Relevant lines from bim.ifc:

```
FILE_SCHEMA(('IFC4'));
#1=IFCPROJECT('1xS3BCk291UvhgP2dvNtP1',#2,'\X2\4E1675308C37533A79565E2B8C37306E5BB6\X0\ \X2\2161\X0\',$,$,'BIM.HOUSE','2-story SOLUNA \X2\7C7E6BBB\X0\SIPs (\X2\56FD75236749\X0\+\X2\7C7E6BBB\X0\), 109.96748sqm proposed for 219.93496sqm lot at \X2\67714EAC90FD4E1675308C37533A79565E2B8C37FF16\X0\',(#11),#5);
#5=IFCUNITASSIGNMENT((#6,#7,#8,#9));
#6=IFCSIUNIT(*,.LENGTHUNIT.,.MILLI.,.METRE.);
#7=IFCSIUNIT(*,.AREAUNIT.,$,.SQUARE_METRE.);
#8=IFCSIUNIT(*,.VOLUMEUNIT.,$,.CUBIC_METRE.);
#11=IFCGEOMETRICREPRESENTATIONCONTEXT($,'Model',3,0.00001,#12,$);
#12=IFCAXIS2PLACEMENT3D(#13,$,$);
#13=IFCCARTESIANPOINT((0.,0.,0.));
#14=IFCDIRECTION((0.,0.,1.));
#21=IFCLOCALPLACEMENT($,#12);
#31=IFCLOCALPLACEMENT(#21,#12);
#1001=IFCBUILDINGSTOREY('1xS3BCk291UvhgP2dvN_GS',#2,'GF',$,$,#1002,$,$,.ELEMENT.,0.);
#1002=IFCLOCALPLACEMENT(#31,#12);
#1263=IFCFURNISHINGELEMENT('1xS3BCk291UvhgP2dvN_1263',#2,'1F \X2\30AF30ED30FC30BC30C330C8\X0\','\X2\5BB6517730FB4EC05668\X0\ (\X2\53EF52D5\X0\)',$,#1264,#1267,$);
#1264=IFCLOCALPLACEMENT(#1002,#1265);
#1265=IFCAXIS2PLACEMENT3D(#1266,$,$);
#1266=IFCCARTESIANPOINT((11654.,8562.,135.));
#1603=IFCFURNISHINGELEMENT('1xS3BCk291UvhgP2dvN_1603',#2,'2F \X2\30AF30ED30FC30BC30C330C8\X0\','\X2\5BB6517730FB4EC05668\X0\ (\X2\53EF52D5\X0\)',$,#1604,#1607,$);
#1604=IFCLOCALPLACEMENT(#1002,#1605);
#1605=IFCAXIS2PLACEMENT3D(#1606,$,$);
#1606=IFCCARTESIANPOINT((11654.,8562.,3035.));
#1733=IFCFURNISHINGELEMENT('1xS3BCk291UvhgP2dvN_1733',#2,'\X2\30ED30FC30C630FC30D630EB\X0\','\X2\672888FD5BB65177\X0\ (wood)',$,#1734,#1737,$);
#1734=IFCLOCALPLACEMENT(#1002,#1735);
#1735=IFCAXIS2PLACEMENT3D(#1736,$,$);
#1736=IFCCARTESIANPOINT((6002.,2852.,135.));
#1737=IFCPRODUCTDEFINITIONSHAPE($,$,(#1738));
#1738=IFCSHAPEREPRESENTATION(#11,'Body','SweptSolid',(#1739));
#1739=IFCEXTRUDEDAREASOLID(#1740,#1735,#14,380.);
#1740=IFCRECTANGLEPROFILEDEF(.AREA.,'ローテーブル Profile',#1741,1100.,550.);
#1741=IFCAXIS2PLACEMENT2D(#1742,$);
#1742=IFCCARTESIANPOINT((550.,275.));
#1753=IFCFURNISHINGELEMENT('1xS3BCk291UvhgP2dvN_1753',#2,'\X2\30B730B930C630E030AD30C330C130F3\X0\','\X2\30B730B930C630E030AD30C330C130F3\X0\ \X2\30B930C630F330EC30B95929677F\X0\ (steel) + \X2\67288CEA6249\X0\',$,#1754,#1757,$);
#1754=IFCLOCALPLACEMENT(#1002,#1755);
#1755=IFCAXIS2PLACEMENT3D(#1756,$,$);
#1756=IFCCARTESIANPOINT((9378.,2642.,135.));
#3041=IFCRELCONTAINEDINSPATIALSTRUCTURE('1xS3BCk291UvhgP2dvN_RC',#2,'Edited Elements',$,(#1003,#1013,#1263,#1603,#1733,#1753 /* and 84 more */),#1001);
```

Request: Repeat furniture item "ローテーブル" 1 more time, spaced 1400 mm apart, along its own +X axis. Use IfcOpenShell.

```python
import ifcopenshell
import ifcopenshell.api.geometry
import ifcopenshell.api.root
import ifcopenshell.util.element
import ifcopenshell.util.placement
import ifcopenshell.util.unit

model = ifcopenshell.open("bim.ifc")
unit_scale = ifcopenshell.util.unit.calculate_unit_scale(model)


def reuse_history(source, copy):
    """copy_class also copies each property set's owner history, people and application; keep the originals."""
    for rel in copy.IsDefinedBy:
        if rel.is_a("IfcRelDefinesByProperties") and (history := rel.RelatingPropertyDefinition.OwnerHistory):
            rel.RelatingPropertyDefinition.OwnerHistory = source.OwnerHistory
            ifcopenshell.util.element.remove_deep2(model, history)


source = model.by_id(1733)
base = ifcopenshell.util.placement.get_local_placement(source.ObjectPlacement)
step = base[:3, 0] * 1.4 / unit_scale

for i in range(1, 2):
    copy = ifcopenshell.api.root.copy_class(model, product=source)
    copy.Representation = ifcopenshell.util.element.copy_deep(
        model, source.Representation, exclude=["IfcGeometricRepresentationContext", "IfcRepresentationMap"]
    )
    reuse_history(source, copy)
    matrix = base.copy()
    matrix[:3, 3] += i * step
    print("added at", matrix[:3, 3].round(3) + 0.0)
    ifcopenshell.api.geometry.edit_object_placement(model, product=copy, matrix=matrix, is_si=False)

model.write("bim_rev.ifc")
```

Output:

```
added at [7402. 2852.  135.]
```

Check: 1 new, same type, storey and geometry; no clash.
